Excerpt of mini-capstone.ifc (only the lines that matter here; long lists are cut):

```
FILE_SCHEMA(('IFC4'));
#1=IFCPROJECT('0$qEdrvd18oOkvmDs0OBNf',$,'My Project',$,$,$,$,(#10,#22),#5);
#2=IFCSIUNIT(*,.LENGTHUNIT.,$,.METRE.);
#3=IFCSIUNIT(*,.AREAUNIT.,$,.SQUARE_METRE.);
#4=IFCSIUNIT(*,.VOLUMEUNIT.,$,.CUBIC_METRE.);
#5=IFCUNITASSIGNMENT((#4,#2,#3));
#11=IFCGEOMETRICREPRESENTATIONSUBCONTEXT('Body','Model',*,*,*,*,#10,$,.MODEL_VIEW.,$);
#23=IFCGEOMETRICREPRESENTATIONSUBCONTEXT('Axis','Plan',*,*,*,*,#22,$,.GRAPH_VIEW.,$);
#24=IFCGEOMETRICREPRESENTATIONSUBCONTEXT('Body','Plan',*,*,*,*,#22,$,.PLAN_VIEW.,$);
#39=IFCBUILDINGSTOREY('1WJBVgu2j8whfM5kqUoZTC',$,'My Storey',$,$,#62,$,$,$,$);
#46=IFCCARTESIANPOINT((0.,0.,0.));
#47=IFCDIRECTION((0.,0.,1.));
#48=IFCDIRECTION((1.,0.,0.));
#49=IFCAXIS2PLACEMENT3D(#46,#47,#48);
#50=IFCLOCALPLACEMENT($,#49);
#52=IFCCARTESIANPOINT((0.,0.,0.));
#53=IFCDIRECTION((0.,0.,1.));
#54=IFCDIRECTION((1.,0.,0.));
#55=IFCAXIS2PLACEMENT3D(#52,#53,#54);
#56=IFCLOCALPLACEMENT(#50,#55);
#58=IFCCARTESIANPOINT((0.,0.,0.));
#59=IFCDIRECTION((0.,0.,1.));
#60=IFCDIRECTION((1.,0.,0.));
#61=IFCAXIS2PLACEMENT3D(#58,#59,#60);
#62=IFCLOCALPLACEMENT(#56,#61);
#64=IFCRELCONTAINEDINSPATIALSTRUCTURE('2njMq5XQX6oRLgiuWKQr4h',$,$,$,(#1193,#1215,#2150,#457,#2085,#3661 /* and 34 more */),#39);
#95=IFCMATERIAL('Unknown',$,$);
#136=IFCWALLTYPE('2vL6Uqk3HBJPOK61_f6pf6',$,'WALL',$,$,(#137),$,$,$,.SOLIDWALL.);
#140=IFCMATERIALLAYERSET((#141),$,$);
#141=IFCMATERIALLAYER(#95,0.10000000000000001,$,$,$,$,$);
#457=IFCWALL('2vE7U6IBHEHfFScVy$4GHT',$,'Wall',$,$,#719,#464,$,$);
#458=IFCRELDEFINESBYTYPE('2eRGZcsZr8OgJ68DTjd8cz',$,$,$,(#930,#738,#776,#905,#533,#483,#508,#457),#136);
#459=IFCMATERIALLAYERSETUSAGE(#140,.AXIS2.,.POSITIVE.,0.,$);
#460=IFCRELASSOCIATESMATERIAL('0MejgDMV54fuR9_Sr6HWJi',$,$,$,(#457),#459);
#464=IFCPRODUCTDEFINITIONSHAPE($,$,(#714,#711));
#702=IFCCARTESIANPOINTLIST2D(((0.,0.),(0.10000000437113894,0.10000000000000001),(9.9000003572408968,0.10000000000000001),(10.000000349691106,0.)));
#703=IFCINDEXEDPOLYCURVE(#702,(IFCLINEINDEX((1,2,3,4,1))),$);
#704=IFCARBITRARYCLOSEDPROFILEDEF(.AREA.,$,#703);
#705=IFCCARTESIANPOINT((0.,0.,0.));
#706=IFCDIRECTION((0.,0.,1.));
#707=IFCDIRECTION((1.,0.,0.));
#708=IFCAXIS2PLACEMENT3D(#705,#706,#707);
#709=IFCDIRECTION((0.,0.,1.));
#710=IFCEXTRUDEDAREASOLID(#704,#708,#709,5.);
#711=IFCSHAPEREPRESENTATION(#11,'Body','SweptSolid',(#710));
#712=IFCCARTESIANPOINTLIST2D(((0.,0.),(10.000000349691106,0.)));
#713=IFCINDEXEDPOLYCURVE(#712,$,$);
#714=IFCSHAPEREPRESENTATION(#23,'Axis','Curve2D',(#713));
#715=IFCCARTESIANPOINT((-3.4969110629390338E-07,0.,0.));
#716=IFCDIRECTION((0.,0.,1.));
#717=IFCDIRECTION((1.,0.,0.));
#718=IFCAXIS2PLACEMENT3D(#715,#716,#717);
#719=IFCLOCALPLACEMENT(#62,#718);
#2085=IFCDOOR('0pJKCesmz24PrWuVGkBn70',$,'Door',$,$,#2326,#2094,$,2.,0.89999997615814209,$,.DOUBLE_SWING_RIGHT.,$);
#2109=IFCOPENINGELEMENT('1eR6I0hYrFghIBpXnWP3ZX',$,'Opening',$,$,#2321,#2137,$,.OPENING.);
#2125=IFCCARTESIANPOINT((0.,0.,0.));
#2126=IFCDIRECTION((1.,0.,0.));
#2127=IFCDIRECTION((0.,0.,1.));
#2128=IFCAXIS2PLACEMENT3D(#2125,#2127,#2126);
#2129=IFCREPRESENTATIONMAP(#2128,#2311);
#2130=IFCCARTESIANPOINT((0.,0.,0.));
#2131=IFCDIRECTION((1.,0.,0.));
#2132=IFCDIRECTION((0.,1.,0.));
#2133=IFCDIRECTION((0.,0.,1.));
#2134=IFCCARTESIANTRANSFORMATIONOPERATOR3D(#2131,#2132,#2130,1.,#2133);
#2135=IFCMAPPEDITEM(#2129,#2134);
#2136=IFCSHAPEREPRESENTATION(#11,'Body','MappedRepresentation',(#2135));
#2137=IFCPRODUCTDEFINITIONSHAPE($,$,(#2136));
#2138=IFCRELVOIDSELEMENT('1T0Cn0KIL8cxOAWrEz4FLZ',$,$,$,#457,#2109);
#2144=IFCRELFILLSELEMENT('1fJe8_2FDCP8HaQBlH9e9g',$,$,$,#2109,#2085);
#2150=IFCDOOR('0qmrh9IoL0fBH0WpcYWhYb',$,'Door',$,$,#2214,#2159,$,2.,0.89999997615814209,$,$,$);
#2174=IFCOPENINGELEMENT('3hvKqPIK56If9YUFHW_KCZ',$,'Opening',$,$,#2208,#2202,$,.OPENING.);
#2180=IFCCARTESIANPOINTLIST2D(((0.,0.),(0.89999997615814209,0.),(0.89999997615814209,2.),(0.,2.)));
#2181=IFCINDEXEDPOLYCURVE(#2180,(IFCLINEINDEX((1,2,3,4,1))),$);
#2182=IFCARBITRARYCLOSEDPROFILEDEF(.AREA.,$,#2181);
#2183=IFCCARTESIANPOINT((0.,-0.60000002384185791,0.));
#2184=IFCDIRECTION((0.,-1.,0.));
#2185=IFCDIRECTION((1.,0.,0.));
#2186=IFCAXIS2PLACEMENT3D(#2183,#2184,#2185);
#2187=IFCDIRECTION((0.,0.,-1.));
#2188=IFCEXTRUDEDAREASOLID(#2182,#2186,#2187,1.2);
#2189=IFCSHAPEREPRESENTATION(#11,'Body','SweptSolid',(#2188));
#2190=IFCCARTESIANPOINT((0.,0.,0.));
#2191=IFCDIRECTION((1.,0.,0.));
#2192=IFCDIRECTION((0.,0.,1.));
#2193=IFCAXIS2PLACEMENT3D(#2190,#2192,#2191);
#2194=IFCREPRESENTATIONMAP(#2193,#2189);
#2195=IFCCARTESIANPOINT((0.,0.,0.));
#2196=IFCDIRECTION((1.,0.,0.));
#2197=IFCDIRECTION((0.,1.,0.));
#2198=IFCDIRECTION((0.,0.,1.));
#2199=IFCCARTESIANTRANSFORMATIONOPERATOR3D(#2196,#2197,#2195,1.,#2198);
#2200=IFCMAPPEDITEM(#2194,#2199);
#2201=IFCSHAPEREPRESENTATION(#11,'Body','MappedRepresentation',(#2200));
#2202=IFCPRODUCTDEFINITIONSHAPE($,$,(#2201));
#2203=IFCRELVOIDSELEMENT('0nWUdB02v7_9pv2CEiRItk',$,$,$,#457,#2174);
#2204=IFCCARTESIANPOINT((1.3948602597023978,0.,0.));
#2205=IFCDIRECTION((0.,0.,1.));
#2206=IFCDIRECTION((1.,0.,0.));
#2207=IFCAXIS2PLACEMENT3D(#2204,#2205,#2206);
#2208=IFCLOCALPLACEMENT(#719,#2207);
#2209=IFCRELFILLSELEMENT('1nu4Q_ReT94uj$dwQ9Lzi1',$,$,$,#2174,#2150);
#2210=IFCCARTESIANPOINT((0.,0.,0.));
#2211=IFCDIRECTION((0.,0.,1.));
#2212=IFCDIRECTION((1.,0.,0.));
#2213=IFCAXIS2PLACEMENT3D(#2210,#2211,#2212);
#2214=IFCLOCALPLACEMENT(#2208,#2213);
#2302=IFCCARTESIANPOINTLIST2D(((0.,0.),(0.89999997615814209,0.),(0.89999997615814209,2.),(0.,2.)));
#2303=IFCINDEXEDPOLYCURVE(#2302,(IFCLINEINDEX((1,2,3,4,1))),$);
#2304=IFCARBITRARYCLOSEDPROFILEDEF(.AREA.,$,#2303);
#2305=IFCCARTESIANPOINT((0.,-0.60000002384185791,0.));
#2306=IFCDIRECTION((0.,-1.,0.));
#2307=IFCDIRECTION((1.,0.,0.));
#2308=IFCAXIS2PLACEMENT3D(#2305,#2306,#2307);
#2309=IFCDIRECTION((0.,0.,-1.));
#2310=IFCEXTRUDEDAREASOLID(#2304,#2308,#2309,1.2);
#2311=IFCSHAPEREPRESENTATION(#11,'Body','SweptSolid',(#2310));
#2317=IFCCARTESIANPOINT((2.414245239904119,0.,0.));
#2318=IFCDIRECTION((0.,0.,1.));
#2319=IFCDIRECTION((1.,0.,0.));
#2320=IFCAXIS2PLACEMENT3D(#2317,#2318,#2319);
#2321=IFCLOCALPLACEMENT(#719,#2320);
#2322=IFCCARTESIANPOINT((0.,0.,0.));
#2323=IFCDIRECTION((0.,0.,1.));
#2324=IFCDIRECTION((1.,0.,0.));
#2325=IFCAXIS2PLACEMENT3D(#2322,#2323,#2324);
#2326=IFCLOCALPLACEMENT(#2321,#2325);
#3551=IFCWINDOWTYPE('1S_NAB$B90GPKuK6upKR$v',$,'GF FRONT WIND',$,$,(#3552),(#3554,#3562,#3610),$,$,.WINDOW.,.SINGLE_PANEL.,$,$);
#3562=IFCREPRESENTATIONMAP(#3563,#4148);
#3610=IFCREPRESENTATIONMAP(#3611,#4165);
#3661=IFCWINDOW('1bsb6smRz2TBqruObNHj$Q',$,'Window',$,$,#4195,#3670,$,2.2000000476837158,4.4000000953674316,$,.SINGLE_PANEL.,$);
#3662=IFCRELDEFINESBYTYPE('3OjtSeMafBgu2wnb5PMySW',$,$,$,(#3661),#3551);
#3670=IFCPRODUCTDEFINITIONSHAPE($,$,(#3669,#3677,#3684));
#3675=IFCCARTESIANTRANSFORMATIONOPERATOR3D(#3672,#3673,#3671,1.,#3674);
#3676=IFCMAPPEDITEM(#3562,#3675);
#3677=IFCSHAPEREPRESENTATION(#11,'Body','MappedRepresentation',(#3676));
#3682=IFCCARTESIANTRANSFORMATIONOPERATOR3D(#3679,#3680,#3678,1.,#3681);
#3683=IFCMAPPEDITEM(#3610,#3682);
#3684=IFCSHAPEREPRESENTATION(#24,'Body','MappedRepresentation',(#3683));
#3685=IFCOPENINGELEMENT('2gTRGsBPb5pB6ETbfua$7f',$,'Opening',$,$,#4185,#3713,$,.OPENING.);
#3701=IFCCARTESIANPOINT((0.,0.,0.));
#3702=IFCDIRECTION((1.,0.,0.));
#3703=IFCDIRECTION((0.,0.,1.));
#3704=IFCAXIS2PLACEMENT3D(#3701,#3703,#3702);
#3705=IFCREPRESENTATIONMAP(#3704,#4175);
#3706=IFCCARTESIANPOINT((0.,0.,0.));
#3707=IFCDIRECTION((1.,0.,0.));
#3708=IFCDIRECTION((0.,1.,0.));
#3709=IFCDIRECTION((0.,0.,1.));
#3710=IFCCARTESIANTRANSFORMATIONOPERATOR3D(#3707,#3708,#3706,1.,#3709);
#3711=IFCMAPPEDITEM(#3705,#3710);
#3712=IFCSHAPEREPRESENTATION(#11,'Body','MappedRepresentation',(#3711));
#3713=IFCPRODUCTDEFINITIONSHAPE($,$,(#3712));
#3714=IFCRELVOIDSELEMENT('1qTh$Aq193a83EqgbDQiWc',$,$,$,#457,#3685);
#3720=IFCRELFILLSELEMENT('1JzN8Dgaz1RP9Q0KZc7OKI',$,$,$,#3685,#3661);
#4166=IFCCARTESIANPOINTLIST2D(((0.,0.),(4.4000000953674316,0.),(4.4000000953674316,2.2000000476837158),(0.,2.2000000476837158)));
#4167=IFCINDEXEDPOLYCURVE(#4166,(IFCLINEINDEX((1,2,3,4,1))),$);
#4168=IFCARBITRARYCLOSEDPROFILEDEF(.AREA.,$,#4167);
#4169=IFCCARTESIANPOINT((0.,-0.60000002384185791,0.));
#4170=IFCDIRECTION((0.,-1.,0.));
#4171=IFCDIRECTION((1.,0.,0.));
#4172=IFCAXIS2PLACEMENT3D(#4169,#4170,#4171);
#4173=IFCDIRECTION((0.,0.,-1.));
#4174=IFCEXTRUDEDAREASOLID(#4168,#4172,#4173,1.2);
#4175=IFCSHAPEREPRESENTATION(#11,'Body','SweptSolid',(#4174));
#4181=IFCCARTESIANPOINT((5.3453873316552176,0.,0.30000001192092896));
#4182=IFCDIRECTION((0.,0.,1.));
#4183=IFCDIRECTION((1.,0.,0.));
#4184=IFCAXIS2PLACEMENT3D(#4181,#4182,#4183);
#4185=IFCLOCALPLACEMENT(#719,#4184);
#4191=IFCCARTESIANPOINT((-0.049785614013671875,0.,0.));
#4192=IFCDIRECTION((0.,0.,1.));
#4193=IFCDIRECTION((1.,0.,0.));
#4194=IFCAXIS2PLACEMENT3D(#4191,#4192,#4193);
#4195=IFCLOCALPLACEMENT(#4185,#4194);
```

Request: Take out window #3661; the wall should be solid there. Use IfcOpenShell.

```python
import ifcopenshell
import ifcopenshell.api.feature
import ifcopenshell.api.root
import ifcopenshell.geom
import ifcopenshell.util.shape

model = ifcopenshell.open("mini-capstone.ifc")
settings = ifcopenshell.geom.settings()


def volume(element):
    """Net volume in cubic metres, openings subtracted."""
    shape = ifcopenshell.geom.create_shape(settings, element)
    return ifcopenshell.util.shape.get_volume(shape.geometry)


window = model.by_guid("1bsb6smRz2TBqruObNHj$Q")
opening = window.FillsVoids[0].RelatingOpeningElement
wall = opening.VoidsElements[0].RelatingBuildingElement
before = volume(wall)

ifcopenshell.api.root.remove_product(model, product=window)
ifcopenshell.api.feature.remove_feature(model, feature=opening)

after = volume(wall)

print(f"wall volume {before:.3f} -> {after:.3f} m3")

model.write("mini-capstone_rev.ifc")
```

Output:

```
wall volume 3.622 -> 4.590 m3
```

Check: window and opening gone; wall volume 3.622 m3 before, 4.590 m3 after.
